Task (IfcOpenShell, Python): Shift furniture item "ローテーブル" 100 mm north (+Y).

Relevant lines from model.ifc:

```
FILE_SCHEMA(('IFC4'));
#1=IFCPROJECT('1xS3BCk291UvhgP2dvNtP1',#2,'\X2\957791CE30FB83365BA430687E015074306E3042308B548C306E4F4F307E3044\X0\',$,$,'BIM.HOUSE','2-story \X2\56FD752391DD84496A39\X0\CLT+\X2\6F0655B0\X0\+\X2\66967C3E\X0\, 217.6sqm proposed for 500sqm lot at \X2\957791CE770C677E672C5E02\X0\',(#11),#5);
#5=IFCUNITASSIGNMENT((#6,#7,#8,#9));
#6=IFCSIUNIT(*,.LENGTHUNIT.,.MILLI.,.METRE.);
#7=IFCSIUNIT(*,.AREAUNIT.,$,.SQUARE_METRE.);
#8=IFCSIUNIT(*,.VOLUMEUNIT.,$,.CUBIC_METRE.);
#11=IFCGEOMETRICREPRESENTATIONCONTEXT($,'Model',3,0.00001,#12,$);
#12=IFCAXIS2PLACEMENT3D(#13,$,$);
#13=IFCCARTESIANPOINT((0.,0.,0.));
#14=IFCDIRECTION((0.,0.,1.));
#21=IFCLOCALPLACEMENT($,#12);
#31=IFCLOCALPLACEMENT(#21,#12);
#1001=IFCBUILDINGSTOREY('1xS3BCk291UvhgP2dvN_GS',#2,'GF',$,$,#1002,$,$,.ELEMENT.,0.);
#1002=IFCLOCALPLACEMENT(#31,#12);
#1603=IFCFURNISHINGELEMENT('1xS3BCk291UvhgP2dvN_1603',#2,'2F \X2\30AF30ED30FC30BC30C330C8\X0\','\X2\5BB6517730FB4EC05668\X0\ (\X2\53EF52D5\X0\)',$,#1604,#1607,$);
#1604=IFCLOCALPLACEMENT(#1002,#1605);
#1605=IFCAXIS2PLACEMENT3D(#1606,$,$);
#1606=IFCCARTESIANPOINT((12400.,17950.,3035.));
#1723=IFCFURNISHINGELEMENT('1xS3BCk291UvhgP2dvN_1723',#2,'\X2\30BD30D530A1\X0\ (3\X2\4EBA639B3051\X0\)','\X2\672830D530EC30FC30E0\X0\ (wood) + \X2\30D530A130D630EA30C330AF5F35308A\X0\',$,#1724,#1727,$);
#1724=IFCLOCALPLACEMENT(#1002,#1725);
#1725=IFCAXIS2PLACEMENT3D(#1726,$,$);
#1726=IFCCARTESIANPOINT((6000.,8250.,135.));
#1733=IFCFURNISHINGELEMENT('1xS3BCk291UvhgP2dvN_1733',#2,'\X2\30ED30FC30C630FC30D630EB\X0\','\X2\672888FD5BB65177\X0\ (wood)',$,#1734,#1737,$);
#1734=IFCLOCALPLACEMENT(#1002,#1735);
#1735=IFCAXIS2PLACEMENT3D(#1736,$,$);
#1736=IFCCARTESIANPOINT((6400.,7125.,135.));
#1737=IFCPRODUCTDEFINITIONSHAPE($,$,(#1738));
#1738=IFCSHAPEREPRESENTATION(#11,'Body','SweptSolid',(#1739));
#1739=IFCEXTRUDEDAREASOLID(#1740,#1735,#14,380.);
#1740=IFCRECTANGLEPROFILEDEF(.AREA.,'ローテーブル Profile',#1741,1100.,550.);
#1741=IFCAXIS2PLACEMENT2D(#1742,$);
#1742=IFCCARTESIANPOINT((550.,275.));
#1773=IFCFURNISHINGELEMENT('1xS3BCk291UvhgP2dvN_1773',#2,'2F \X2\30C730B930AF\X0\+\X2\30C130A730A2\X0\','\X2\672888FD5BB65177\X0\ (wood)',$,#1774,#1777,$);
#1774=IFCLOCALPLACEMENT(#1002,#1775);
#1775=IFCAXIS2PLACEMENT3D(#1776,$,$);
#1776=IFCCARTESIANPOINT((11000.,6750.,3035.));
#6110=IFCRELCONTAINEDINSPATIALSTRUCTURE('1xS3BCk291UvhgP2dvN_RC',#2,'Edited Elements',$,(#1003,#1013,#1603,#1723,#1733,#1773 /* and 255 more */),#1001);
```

```python
import ifcopenshell
import ifcopenshell.api.geometry
import ifcopenshell.util.placement
import ifcopenshell.util.unit

model = ifcopenshell.open("model.ifc")
unit_scale = ifcopenshell.util.unit.calculate_unit_scale(model)

item = model.by_guid("1xS3BCk291UvhgP2dvN_1733")
matrix = ifcopenshell.util.placement.get_local_placement(item.ObjectPlacement)
matrix[1, 3] += 0.1 / unit_scale
ifcopenshell.api.geometry.edit_object_placement(model, product=item, matrix=matrix, is_si=False)

print(ifcopenshell.util.placement.get_local_placement(item.ObjectPlacement).round(3) + 0.0)

model.write("model_rev.ifc")
```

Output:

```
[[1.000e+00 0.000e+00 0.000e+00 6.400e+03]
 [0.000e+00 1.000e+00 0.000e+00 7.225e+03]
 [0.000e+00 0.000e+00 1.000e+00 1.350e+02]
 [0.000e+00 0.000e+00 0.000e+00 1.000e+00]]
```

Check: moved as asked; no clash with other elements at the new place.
